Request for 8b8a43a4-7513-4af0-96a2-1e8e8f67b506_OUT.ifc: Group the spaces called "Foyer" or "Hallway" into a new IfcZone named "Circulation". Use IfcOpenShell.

First a look at what the model holds.

```python
import ifcopenshell

model = ifcopenshell.open("8b8a43a4-7513-4af0-96a2-1e8e8f67b506_OUT.ifc")
print(model.schema)
seen = {}
for space in model.by_type("IfcSpace"):
    seen[space.LongName] = seen.get(space.LongName, 0) + 1
for name, count in sorted(seen.items(), key=str):
    print(count, "x", name)
print("zones:", [z.Name for z in model.by_type("IfcZone")][:20])
```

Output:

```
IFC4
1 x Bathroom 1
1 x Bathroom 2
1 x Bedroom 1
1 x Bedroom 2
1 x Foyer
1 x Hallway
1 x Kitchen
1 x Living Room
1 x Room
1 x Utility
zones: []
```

```python
import ifcopenshell
import ifcopenshell.api.group
import ifcopenshell.api.root

model = ifcopenshell.open("8b8a43a4-7513-4af0-96a2-1e8e8f67b506_OUT.ifc")

names = {"Foyer", "Hallway"}
spaces = [s for s in model.by_type("IfcSpace") if s.LongName in names]

zone = ifcopenshell.api.root.create_entity(model, ifc_class="IfcZone", name="Circulation")
ifcopenshell.api.group.assign_group(model, products=spaces, group=zone)
print(len(spaces), "spaces in", zone.Name)

model.write("8b8a43a4-7513-4af0-96a2-1e8e8f67b506_OUT_updated.ifc")
```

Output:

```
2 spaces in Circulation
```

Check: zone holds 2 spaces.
